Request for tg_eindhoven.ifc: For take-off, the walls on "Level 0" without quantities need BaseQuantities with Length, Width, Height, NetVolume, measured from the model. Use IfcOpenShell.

First a look at what the model holds.

```python
import ifcopenshell
import ifcopenshell.util.element
import ifcopenshell.util.unit

model = ifcopenshell.open("tg_eindhoven.ifc")
print(model.schema)
for unit_type in ("LENGTHUNIT", "AREAUNIT", "VOLUMEUNIT"):
    print(unit_type, ifcopenshell.util.unit.calculate_unit_scale(model, unit_type))
storey = next(s for s in model.by_type("IfcBuildingStorey") if s.Name == "Level 0")
walls = [e for e in ifcopenshell.util.element.get_decomposition(storey) if e.is_a("IfcWall")]
for e in sorted(walls, key=lambda e: e.id()):
    print(e.id(), e.is_a(), e.Name, list(ifcopenshell.util.element.get_psets(e, qtos_only=True)), sep=" | ")
```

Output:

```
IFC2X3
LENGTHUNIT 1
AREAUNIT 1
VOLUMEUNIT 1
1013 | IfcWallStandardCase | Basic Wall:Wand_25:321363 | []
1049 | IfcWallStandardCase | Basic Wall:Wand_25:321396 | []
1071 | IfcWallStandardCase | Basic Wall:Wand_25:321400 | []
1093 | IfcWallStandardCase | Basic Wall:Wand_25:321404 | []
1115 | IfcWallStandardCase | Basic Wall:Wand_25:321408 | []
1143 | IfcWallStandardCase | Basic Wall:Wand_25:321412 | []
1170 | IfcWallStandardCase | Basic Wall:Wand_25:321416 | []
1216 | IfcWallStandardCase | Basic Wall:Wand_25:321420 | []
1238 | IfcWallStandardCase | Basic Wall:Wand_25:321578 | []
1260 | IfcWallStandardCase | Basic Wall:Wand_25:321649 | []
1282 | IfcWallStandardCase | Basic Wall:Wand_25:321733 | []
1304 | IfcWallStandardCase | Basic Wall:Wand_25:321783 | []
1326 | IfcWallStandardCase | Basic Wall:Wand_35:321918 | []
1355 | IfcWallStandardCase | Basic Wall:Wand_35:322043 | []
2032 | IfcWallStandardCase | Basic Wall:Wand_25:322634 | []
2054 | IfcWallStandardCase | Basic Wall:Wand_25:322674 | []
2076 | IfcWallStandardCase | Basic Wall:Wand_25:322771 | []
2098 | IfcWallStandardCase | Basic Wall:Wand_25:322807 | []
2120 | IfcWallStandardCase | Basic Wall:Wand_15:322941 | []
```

```python
import ifcopenshell
import ifcopenshell.api.pset
import ifcopenshell.geom
import ifcopenshell.util.element
import ifcopenshell.util.shape
import ifcopenshell.util.unit

model = ifcopenshell.open("tg_eindhoven.ifc")
unit_scale = ifcopenshell.util.unit.calculate_unit_scale(model)
volume_scale = ifcopenshell.util.unit.calculate_unit_scale(model, "VOLUMEUNIT")
settings = ifcopenshell.geom.settings()

storey = next(s for s in model.by_type("IfcBuildingStorey") if s.Name == "Level 0")
walls = [e for e in ifcopenshell.util.element.get_decomposition(storey) if e.is_a("IfcWall")]

for e in sorted(walls, key=lambda e: e.id()):
    if ifcopenshell.util.element.get_psets(e, qtos_only=True, should_inherit=False):
        continue
    # Geometry comes back in metres, in the element's own axes.
    shape = ifcopenshell.geom.create_shape(settings, e)
    values = {
        "Length": ifcopenshell.util.shape.get_x(shape.geometry) / unit_scale,
        "Width": ifcopenshell.util.shape.get_y(shape.geometry) / unit_scale,
        "Height": ifcopenshell.util.shape.get_z(shape.geometry) / unit_scale,
        "NetVolume": ifcopenshell.util.shape.get_volume(shape.geometry) / volume_scale,
    }
    qto = ifcopenshell.api.pset.add_qto(model, product=e, name="BaseQuantities")
    ifcopenshell.api.pset.edit_qto(model, qto=qto, properties=values)
    print(e.id(), {k: round(v, 3) for k, v in values.items()})

model.write("tg_eindhoven_rev.ifc")
```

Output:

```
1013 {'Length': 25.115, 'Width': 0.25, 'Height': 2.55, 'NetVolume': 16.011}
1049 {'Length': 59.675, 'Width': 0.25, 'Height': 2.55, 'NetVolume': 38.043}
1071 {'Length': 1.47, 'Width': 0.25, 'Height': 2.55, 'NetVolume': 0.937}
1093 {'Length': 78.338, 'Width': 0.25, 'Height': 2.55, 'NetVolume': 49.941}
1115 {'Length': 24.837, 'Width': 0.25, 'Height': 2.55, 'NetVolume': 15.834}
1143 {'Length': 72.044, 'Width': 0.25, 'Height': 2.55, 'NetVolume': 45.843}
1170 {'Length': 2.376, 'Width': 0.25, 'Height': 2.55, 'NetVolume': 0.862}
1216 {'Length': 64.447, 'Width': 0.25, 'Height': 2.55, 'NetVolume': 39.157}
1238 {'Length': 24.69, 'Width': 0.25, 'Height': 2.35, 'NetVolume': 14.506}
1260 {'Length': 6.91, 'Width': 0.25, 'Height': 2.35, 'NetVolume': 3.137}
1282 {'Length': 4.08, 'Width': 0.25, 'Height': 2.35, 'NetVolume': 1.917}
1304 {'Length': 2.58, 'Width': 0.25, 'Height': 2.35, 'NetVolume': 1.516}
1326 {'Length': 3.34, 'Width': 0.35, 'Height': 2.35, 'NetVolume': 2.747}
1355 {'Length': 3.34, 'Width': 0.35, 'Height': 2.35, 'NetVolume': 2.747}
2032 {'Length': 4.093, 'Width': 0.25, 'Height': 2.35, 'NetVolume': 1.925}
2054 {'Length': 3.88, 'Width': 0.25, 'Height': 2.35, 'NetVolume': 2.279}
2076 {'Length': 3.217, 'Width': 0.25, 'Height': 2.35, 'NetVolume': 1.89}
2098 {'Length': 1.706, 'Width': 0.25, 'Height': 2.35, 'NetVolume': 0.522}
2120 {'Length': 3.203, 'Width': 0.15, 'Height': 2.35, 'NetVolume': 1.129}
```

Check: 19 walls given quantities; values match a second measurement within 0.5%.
